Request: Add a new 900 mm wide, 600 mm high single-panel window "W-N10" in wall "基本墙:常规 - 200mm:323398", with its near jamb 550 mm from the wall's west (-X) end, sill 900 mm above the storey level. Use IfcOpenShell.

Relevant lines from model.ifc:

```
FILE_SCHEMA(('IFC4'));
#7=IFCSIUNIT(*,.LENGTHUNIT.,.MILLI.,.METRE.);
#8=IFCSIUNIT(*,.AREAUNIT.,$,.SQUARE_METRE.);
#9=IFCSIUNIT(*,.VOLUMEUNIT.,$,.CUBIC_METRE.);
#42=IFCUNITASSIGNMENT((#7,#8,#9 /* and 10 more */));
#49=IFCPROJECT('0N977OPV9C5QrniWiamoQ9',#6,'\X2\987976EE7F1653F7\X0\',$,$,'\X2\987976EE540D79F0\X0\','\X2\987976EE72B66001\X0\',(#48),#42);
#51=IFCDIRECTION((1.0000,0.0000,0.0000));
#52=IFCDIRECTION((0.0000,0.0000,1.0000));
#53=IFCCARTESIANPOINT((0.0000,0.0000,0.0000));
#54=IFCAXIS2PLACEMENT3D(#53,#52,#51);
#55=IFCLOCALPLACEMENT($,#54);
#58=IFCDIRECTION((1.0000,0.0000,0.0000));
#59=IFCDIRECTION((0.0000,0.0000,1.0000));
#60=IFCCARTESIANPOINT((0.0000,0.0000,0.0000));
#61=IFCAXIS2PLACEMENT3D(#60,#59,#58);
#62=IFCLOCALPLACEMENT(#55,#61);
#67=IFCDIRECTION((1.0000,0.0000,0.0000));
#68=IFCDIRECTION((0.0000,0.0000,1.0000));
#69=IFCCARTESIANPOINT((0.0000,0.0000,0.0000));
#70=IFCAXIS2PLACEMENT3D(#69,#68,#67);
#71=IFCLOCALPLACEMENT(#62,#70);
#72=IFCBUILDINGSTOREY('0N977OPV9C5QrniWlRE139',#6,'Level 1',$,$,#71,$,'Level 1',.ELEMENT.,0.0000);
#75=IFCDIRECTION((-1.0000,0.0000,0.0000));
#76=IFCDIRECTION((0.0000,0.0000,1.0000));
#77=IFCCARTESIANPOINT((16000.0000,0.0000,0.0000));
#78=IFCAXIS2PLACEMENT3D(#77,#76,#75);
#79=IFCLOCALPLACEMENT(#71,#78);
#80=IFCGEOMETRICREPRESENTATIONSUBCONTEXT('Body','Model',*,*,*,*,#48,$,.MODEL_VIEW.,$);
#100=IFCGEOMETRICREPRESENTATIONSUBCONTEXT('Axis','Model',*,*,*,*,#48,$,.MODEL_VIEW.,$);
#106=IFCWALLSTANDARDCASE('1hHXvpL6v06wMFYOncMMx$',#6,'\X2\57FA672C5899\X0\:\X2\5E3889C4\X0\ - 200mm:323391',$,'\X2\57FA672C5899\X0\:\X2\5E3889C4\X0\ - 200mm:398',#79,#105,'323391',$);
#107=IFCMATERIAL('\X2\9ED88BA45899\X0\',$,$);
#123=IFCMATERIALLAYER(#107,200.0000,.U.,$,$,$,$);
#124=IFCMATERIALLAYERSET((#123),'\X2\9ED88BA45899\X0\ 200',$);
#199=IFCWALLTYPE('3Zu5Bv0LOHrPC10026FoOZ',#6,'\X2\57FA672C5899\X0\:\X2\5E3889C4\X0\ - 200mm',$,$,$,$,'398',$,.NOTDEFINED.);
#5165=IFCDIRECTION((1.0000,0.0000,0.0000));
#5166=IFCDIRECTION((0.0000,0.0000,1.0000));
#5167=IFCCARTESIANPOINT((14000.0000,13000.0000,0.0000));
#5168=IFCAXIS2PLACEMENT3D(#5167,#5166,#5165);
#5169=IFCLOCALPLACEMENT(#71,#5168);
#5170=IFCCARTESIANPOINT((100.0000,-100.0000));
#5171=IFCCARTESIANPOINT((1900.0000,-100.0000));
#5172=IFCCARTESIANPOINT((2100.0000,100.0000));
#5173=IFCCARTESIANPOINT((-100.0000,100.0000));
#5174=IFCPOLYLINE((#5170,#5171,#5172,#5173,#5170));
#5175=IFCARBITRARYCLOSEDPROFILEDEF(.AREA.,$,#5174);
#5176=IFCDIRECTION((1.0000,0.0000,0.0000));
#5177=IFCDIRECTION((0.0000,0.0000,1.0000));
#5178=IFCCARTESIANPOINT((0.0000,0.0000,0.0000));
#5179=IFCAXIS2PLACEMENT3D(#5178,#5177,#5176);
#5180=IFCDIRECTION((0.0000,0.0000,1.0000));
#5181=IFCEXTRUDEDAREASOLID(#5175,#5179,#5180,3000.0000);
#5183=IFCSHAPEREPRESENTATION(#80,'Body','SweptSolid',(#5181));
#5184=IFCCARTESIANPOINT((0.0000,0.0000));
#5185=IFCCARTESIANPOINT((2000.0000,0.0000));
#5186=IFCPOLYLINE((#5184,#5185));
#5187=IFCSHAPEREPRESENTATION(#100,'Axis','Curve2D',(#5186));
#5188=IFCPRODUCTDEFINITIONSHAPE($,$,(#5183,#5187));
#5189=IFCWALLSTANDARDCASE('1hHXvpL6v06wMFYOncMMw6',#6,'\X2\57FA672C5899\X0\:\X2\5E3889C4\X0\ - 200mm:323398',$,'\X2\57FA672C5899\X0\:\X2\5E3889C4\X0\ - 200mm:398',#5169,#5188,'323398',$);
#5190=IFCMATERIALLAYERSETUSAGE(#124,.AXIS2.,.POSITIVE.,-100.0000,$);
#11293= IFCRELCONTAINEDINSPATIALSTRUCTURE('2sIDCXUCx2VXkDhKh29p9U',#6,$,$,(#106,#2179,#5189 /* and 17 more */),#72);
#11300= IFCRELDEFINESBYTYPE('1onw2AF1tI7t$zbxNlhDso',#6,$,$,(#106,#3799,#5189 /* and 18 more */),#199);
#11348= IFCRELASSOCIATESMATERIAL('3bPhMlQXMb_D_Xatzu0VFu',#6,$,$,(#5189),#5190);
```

```python
import numpy as np
import ifcopenshell
import ifcopenshell.api.feature
import ifcopenshell.api.geometry
import ifcopenshell.api.root
import ifcopenshell.api.spatial
import ifcopenshell.geom
import ifcopenshell.util.element
import ifcopenshell.util.placement
import ifcopenshell.util.representation
import ifcopenshell.util.shape
import ifcopenshell.util.unit

model = ifcopenshell.open("model.ifc")
unit_scale = ifcopenshell.util.unit.calculate_unit_scale(model)
settings = ifcopenshell.geom.settings()


def volume(element):
    """Net volume in cubic metres, openings subtracted."""
    shape = ifcopenshell.geom.create_shape(settings, element)
    return ifcopenshell.util.shape.get_volume(shape.geometry)


wall = model.by_guid("1hHXvpL6v06wMFYOncMMw6")
storey = ifcopenshell.util.element.get_container(wall, ifc_class="IfcBuildingStorey")
context = ifcopenshell.util.representation.get_context(model, "Model", "Body", "MODEL_VIEW")
before = volume(wall)

width, height, from_end, sill = 0.9, 0.6, 0.55, 0.9  # metres

# The wall runs along its own X axis, and the end named is its -X end.
wall_shape = ifcopenshell.geom.create_shape(settings, wall)
x, y, z = ifcopenshell.util.shape.get_vertices(wall_shape.geometry).T
start = x.min() + from_end
face, thickness = float(y.min()), float(y.max() - y.min())
wall_matrix = ifcopenshell.util.placement.get_local_placement(wall.ObjectPlacement)
level = ifcopenshell.util.placement.get_local_placement(storey.ObjectPlacement)[2, 3]


def in_wall(x, y):
    """Placement at x, y metres in the wall's axes, at sill height."""
    matrix = wall_matrix.copy()
    matrix[:, 3] = wall_matrix @ np.array([x / unit_scale, y / unit_scale, 0.0, 1.0])
    matrix[2, 3] = level + sill / unit_scale
    return matrix


# Opening: a box that overshoots both wall faces by 50 mm.
opening = ifcopenshell.api.root.create_entity(model, ifc_class="IfcOpeningElement", predefined_type="OPENING")
box = ifcopenshell.api.geometry.add_wall_representation(
    model, context=context, length=width, height=height, thickness=thickness + 0.1
)
ifcopenshell.api.geometry.assign_representation(model, product=opening, representation=box)
ifcopenshell.api.geometry.edit_object_placement(model, product=opening, matrix=in_wall(start, face - 0.05), is_si=False)
ifcopenshell.api.feature.add_feature(model, feature=opening, element=wall)

window = ifcopenshell.api.root.create_entity(model, ifc_class="IfcWindow", name="W-N10", predefined_type="WINDOW")
window.OverallWidth, window.OverallHeight = width / unit_scale, height / unit_scale
window.PartitioningType = "SINGLE_PANEL"
body = ifcopenshell.api.geometry.add_window_representation(
    model,
    context=context,
    overall_width=window.OverallWidth,
    overall_height=window.OverallHeight,
    partition_type="SINGLE_PANEL",
)
ifcopenshell.api.geometry.assign_representation(model, product=window, representation=body)
ifcopenshell.api.spatial.assign_container(model, products=[window], relating_structure=storey)
ifcopenshell.api.feature.add_filling(model, opening=opening, element=window)

# Centre the window in the wall's thickness.
ifcopenshell.api.geometry.edit_object_placement(model, product=window, matrix=in_wall(start, face), is_si=False)
window_shape = ifcopenshell.geom.create_shape(settings, window)
depth = ifcopenshell.util.shape.get_vertices(window_shape.geometry)[:, 1]
offset = face + thickness / 2 - (depth.min() + depth.max()) / 2
ifcopenshell.api.geometry.edit_object_placement(model, product=window, matrix=in_wall(start, offset), is_si=False)

after = volume(wall)

print(f"wall volume {before:.3f} -> {after:.3f} m3")

model.write("model_updated.ifc")
```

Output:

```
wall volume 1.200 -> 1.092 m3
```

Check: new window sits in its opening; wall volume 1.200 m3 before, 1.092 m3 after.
